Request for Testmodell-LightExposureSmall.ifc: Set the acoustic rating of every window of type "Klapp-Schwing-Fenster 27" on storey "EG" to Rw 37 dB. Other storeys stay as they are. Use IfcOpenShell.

First a look at what the model holds.

```python
import ifcopenshell
import ifcopenshell.util.element

model = ifcopenshell.open("Testmodell-LightExposureSmall.ifc")
print(model.schema)
storey = next(s for s in model.by_type("IfcBuildingStorey") if s.Name == "EG")
windows = [e for e in ifcopenshell.util.element.get_decomposition(storey) if e.is_a("IfcWindow")]
seen = {}
for e in windows:
    element_type = ifcopenshell.util.element.get_type(e)
    key = (element_type.Name if element_type != e and element_type else None, ifcopenshell.util.element.get_pset(e, "Pset_WindowCommon", "AcousticRating"))
    seen[key] = seen.get(key, 0) + 1
for (name, value), count in sorted(seen.items(), key=str):
    print(count, "x", name, "|", value)
```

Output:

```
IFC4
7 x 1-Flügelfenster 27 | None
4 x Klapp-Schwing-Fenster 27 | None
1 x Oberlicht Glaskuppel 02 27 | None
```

```python
import ifcopenshell
import ifcopenshell.api.pset
import ifcopenshell.util.element

model = ifcopenshell.open("Testmodell-LightExposureSmall.ifc")

storey = next(s for s in model.by_type("IfcBuildingStorey") if s.Name == "EG")
windows = [e for e in ifcopenshell.util.element.get_decomposition(storey) if e.is_a("IfcWindow")]

count = 0
for e in windows:
    element_type = ifcopenshell.util.element.get_type(e)
    if element_type in (None, e) or element_type.Name != "Klapp-Schwing-Fenster 27":
        continue
    # add_pset returns the element's existing set when there is one.
    pset = ifcopenshell.api.pset.add_pset(model, product=e, name="Pset_WindowCommon")
    ifcopenshell.api.pset.edit_pset(model, pset=pset, properties={"AcousticRating": "Rw 37 dB"})
    count += 1

print(count, "windows updated")

model.write("Testmodell-LightExposureSmall_updated.ifc")
```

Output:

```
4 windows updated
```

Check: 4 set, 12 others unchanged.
